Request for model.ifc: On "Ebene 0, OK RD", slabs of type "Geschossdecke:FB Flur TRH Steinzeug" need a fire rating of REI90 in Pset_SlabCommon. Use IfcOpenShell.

First a look at what the model holds.

```python
import ifcopenshell
import ifcopenshell.util.element

model = ifcopenshell.open("model.ifc")
print(model.schema)
storey = next(s for s in model.by_type("IfcBuildingStorey") if s.Name == "Ebene 0, OK RD")
slabs = [e for e in ifcopenshell.util.element.get_decomposition(storey) if e.is_a("IfcSlab")]
seen = {}
for e in slabs:
    element_type = ifcopenshell.util.element.get_type(e)
    key = (element_type.Name if element_type != e and element_type else None, ifcopenshell.util.element.get_pset(e, "Pset_SlabCommon", "FireRating"))
    seen[key] = seen.get(key, 0) + 1
for (name, value), count in sorted(seen.items(), key=str):
    print(count, "x", name, "|", value)
```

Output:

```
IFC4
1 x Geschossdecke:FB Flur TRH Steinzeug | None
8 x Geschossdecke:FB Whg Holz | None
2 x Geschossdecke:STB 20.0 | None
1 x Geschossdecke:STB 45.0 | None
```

```python
import ifcopenshell
import ifcopenshell.api.pset
import ifcopenshell.util.element

model = ifcopenshell.open("model.ifc")

storey = next(s for s in model.by_type("IfcBuildingStorey") if s.Name == "Ebene 0, OK RD")
slabs = [e for e in ifcopenshell.util.element.get_decomposition(storey) if e.is_a("IfcSlab")]

count = 0
for e in slabs:
    element_type = ifcopenshell.util.element.get_type(e)
    if element_type in (None, e) or element_type.Name != "Geschossdecke:FB Flur TRH Steinzeug":
        continue
    # add_pset returns the element's existing set when there is one.
    pset = ifcopenshell.api.pset.add_pset(model, product=e, name="Pset_SlabCommon")
    ifcopenshell.api.pset.edit_pset(model, pset=pset, properties={"FireRating": "REI90"})
    count += 1

print(count, "slabs updated")

model.write("model-out.ifc")
```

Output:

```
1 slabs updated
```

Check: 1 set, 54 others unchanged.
